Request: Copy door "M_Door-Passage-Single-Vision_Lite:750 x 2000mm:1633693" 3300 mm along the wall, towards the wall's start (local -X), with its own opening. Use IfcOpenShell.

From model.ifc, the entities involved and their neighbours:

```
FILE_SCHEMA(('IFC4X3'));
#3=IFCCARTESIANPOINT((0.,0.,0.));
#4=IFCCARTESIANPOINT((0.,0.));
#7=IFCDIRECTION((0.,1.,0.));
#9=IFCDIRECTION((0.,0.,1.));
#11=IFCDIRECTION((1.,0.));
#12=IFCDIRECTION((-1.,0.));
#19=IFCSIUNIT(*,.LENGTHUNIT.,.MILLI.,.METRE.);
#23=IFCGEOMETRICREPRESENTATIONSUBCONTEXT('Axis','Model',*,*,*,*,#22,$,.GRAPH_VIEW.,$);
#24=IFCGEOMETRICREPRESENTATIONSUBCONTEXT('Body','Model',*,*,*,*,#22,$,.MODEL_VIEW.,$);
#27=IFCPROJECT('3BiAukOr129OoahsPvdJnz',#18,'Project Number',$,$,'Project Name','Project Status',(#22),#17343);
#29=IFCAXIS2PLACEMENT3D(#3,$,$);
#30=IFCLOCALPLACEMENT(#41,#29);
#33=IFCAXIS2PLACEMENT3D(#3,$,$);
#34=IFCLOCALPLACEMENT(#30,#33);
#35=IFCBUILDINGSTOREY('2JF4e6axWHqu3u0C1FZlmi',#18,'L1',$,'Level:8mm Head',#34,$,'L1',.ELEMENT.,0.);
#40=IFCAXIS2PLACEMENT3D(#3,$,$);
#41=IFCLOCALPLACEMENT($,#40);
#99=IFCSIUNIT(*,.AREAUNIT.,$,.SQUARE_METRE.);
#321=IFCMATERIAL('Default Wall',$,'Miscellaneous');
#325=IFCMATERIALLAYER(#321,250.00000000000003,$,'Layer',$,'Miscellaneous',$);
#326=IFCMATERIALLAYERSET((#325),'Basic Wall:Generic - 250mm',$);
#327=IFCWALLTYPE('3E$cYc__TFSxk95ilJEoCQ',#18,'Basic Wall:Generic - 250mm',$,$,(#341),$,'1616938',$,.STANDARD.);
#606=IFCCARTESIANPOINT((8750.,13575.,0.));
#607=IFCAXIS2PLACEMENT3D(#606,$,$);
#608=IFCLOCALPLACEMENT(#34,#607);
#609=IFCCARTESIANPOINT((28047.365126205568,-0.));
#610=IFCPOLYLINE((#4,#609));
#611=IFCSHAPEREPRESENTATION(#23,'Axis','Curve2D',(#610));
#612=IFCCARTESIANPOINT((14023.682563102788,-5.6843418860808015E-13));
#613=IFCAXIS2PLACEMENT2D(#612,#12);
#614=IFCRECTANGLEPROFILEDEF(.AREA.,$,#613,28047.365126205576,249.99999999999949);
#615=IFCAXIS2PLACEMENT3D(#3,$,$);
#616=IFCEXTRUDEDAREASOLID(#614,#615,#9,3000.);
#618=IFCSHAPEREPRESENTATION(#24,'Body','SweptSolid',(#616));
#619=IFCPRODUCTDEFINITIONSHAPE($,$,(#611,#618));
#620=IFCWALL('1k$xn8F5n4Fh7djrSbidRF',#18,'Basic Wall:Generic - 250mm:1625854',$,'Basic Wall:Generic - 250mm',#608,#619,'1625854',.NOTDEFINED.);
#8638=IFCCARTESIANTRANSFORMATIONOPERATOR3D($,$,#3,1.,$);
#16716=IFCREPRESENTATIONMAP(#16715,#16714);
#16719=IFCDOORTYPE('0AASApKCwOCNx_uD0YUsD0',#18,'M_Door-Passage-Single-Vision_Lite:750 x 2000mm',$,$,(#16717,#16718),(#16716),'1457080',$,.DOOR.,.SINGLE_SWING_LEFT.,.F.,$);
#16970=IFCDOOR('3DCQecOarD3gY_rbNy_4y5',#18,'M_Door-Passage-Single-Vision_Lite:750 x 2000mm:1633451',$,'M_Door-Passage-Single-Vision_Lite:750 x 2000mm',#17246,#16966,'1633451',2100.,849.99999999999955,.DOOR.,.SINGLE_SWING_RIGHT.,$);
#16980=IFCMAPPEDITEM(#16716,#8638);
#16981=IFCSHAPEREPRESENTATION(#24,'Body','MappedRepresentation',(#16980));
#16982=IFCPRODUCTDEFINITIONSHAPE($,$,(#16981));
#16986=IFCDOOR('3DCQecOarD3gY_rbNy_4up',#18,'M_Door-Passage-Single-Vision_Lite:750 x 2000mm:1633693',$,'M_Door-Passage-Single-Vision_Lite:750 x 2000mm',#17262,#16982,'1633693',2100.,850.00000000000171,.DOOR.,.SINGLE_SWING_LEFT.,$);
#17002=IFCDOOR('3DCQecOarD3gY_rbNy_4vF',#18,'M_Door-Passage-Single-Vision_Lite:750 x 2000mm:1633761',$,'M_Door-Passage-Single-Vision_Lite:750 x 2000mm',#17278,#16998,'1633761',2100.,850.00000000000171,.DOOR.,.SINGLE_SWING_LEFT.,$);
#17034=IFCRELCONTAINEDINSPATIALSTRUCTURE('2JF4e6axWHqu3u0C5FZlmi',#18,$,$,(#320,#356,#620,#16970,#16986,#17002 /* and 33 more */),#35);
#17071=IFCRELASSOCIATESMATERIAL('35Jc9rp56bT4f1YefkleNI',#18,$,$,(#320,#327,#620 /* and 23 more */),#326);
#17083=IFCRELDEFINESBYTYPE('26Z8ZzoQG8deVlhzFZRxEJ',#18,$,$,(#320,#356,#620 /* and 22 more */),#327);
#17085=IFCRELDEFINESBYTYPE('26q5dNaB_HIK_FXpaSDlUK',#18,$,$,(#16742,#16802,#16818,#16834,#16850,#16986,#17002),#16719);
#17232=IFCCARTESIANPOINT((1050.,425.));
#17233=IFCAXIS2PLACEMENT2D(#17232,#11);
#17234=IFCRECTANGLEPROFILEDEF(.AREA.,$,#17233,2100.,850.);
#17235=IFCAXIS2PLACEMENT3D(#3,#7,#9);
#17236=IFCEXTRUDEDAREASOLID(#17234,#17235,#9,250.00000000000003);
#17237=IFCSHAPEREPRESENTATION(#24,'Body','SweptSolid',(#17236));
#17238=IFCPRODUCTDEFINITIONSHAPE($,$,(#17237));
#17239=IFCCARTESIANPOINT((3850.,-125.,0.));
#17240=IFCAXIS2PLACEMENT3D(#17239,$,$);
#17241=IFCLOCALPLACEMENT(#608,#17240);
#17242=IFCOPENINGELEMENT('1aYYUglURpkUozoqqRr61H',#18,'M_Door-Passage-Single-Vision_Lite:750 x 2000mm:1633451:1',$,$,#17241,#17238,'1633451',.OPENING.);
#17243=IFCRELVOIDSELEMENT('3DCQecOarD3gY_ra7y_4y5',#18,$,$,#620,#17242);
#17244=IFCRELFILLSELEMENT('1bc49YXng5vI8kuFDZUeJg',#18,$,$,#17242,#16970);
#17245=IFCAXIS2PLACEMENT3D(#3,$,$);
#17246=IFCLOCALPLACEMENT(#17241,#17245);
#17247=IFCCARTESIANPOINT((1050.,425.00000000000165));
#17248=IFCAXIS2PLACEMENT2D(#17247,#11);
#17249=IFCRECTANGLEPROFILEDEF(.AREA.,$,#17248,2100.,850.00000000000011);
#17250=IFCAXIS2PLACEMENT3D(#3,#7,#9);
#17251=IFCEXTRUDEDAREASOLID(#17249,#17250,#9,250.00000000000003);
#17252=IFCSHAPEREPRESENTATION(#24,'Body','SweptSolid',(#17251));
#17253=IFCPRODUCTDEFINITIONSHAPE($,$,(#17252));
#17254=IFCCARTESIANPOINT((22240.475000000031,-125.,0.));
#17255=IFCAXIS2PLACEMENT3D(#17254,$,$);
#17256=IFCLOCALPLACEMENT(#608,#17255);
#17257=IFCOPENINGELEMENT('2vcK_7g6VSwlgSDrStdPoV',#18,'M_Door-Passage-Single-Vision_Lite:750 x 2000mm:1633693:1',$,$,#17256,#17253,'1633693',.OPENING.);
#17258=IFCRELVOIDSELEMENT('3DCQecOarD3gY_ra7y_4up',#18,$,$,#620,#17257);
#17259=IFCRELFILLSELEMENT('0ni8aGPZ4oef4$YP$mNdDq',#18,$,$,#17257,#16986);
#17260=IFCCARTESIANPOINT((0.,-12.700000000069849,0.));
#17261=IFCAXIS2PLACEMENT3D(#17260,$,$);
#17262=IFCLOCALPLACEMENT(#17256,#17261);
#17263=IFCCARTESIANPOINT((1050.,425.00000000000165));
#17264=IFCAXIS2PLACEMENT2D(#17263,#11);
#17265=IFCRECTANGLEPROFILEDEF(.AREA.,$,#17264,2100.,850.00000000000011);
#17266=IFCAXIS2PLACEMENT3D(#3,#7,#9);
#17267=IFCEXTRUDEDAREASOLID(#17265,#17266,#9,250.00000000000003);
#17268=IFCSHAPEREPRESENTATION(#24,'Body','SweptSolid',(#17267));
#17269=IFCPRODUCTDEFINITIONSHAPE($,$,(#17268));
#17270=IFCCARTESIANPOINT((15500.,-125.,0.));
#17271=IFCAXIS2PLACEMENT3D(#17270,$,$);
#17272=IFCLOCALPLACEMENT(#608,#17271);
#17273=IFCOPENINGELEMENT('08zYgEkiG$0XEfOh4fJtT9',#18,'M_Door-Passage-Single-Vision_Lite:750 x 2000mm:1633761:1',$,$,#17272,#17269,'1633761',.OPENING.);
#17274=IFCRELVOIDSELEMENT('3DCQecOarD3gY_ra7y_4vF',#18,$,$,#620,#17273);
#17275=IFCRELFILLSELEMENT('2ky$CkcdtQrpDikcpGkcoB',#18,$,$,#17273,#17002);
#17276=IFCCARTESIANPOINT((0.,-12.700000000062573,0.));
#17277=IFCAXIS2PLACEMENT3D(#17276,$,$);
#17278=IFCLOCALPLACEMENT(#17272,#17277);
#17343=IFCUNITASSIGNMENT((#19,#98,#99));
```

```python
import ifcopenshell
import ifcopenshell.api.feature
import ifcopenshell.api.geometry
import ifcopenshell.api.root
import ifcopenshell.geom
import ifcopenshell.util.element
import ifcopenshell.util.placement
import ifcopenshell.util.shape
import ifcopenshell.util.unit

model = ifcopenshell.open("model.ifc")
unit_scale = ifcopenshell.util.unit.calculate_unit_scale(model)
settings = ifcopenshell.geom.settings()


def volume(element):
    """Net volume in cubic metres, openings subtracted."""
    shape = ifcopenshell.geom.create_shape(settings, element)
    return ifcopenshell.util.shape.get_volume(shape.geometry)


def reuse_history(source, copy):
    """copy_class also copies each property set's owner history, people and application; keep the originals."""
    for rel in copy.IsDefinedBy:
        if rel.is_a("IfcRelDefinesByProperties") and (history := rel.RelatingPropertyDefinition.OwnerHistory):
            rel.RelatingPropertyDefinition.OwnerHistory = source.OwnerHistory
            ifcopenshell.util.element.remove_deep2(model, history)


door = model.by_guid("3DCQecOarD3gY_rbNy_4up")
opening = door.FillsVoids[0].RelatingOpeningElement
wall = opening.VoidsElements[0].RelatingBuildingElement
before = volume(wall)
shift = ifcopenshell.util.placement.get_local_placement(wall.ObjectPlacement)[:3, 0] * -3.3 / unit_scale

# copy_class copies the void relationship, type, container and properties, but no geometry.
new_opening = ifcopenshell.api.root.copy_class(model, product=opening)
new_opening.Representation = ifcopenshell.util.element.copy_deep(
    model, opening.Representation, exclude=["IfcGeometricRepresentationContext", "IfcRepresentationMap"]
)
new_opening.Name = "M_Door-Passage-Single-Vision_Lite:750 x 2000mm"
new_opening.Tag = None
new_door = ifcopenshell.api.root.copy_class(model, product=door)
new_door.Representation = ifcopenshell.util.element.copy_deep(
    model, door.Representation, exclude=["IfcGeometricRepresentationContext", "IfcRepresentationMap"]
)
new_door.Name = "M_Door-Passage-Single-Vision_Lite:750 x 2000mm"
new_door.Tag = None
reuse_history(door, new_door)
ifcopenshell.api.feature.add_filling(model, opening=new_opening, element=new_door)

for old, new in ((opening, new_opening), (door, new_door)):
    matrix = ifcopenshell.util.placement.get_local_placement(old.ObjectPlacement)
    matrix[:3, 3] += shift
    ifcopenshell.api.geometry.edit_object_placement(model, product=new, matrix=matrix, is_si=False)

after = volume(wall)

print(f"wall volume {before:.3f} -> {after:.3f} m3")

model.write("model_v2.ifc")
```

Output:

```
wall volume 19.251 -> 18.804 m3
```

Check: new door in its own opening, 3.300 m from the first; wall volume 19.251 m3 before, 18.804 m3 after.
